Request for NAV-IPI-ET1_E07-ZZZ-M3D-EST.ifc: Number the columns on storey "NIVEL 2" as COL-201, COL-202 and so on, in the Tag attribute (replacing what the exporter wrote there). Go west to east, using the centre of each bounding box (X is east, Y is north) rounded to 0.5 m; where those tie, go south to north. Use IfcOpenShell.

First a look at what the model holds.

```python
import ifcopenshell
import ifcopenshell.util.element
import ifcopenshell.util.placement

model = ifcopenshell.open("NAV-IPI-ET1_E07-ZZZ-M3D-EST.ifc")
print(model.schema)
storey = next(s for s in model.by_type("IfcBuildingStorey") if s.Name == "NIVEL 2")
columns = [e for e in ifcopenshell.util.element.get_decomposition(storey) if e.is_a("IfcColumn")]
for e in sorted(columns, key=lambda e: e.id()):
    origin = ifcopenshell.util.placement.get_local_placement(e.ObjectPlacement)[:3, 3]
    print(e.id(), e.Tag, e.Name, origin.round(2) + 0.0, sep=" | ")
```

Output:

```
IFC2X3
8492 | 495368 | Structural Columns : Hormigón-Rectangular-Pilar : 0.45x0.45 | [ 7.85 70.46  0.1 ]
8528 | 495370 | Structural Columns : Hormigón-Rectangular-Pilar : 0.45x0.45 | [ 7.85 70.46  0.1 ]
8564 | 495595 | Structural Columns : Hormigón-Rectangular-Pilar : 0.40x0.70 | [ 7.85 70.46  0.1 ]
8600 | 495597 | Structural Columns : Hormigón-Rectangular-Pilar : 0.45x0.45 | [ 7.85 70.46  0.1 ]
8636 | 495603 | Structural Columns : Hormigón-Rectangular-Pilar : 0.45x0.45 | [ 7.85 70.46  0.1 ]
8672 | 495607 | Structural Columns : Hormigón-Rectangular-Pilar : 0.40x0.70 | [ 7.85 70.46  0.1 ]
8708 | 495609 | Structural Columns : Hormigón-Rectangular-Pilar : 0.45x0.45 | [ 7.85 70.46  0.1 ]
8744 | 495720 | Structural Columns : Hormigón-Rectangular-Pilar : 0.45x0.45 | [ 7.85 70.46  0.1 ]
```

```python
import ifcopenshell
import ifcopenshell.geom
import ifcopenshell.util.element
import ifcopenshell.util.shape

model = ifcopenshell.open("NAV-IPI-ET1_E07-ZZZ-M3D-EST.ifc")
settings = ifcopenshell.geom.settings()
settings.set("use-world-coords", True)


def centre(element):
    shape = ifcopenshell.geom.create_shape(settings, element)
    return ifcopenshell.util.shape.get_bbox_centroid(shape.geometry)


storey = next(s for s in model.by_type("IfcBuildingStorey") if s.Name == "NIVEL 2")
columns = [e for e in ifcopenshell.util.element.get_decomposition(storey) if e.is_a("IfcColumn")]

# Insertion points can sit at a corner or the storey origin, so sort by the geometry (in metres).
centres = {e: centre(e) for e in columns}
columns.sort(key=lambda e: (round(centres[e][0] / 0.5), centres[e][1]))

for i, e in enumerate(columns, start=1):
    number = f"COL-2{i:02d}"
    e.Tag = number
    print(e.id(), number)

model.write("NAV-IPI-ET1_E07-ZZZ-M3D-EST_rev.ifc")
```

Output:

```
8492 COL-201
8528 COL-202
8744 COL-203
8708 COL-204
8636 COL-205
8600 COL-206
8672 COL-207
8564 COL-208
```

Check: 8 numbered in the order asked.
